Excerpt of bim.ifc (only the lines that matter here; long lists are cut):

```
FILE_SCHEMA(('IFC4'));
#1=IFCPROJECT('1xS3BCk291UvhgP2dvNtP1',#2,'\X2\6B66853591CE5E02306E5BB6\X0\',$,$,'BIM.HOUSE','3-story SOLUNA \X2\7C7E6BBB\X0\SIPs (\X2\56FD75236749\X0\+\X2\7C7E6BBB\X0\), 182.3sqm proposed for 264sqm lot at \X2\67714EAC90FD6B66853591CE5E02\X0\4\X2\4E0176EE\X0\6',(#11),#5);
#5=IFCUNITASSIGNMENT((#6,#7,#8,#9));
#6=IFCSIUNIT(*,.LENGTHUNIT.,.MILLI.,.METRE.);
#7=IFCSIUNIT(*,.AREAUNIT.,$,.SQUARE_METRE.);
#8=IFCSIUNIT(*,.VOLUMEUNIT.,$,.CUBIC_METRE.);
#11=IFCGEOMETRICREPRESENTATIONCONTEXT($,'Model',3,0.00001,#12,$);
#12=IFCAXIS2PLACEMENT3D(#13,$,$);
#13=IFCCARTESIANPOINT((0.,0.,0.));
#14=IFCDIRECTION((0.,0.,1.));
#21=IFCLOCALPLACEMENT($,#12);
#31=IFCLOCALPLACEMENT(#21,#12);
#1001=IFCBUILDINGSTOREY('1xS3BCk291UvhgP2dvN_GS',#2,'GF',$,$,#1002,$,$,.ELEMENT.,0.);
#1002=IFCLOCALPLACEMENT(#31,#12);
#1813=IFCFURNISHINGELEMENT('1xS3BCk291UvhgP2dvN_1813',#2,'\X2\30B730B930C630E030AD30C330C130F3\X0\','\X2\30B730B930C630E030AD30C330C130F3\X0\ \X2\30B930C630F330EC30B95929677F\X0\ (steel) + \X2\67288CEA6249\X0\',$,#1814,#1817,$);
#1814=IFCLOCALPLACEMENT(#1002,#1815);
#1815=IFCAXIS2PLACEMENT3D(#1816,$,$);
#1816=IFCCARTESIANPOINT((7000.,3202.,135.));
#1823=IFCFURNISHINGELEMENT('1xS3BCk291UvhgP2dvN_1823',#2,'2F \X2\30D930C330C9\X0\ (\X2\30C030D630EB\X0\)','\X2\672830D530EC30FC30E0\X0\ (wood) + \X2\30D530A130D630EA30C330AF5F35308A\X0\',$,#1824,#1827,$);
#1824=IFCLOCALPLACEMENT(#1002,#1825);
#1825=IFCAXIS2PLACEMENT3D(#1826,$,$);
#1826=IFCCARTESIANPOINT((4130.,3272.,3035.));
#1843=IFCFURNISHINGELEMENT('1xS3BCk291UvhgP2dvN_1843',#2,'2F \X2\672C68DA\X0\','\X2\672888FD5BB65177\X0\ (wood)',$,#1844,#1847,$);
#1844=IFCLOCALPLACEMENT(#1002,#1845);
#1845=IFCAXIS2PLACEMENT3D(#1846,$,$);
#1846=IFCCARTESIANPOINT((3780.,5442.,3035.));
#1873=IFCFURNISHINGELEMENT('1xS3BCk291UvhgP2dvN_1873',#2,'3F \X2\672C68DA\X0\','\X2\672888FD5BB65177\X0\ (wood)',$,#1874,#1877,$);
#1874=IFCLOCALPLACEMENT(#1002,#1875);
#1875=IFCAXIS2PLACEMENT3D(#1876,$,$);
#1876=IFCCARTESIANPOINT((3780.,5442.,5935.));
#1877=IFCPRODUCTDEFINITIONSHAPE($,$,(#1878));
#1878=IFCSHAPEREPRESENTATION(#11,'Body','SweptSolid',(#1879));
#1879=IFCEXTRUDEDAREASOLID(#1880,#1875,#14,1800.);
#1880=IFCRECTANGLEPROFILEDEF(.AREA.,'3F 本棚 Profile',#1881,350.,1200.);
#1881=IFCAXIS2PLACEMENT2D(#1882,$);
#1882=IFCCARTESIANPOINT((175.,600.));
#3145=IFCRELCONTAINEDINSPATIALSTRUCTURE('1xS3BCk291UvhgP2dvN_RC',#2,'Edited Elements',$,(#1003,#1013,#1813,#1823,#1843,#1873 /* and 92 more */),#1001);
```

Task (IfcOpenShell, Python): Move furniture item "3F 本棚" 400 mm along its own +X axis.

```python
import ifcopenshell
import ifcopenshell.api.geometry
import ifcopenshell.util.placement
import ifcopenshell.util.unit

model = ifcopenshell.open("bim.ifc")
unit_scale = ifcopenshell.util.unit.calculate_unit_scale(model)

item = model.by_guid("1xS3BCk291UvhgP2dvN_1873")
matrix = ifcopenshell.util.placement.get_local_placement(item.ObjectPlacement)
matrix[:3, 3] += matrix[:3, 0] * 0.4 / unit_scale
ifcopenshell.api.geometry.edit_object_placement(model, product=item, matrix=matrix, is_si=False)

print(ifcopenshell.util.placement.get_local_placement(item.ObjectPlacement).round(3) + 0.0)

model.write("bim_updated.ifc")
```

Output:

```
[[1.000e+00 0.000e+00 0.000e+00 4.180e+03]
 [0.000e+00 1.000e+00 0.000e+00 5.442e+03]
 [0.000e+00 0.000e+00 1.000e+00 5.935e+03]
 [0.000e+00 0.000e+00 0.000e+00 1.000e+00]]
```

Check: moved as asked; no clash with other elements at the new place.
